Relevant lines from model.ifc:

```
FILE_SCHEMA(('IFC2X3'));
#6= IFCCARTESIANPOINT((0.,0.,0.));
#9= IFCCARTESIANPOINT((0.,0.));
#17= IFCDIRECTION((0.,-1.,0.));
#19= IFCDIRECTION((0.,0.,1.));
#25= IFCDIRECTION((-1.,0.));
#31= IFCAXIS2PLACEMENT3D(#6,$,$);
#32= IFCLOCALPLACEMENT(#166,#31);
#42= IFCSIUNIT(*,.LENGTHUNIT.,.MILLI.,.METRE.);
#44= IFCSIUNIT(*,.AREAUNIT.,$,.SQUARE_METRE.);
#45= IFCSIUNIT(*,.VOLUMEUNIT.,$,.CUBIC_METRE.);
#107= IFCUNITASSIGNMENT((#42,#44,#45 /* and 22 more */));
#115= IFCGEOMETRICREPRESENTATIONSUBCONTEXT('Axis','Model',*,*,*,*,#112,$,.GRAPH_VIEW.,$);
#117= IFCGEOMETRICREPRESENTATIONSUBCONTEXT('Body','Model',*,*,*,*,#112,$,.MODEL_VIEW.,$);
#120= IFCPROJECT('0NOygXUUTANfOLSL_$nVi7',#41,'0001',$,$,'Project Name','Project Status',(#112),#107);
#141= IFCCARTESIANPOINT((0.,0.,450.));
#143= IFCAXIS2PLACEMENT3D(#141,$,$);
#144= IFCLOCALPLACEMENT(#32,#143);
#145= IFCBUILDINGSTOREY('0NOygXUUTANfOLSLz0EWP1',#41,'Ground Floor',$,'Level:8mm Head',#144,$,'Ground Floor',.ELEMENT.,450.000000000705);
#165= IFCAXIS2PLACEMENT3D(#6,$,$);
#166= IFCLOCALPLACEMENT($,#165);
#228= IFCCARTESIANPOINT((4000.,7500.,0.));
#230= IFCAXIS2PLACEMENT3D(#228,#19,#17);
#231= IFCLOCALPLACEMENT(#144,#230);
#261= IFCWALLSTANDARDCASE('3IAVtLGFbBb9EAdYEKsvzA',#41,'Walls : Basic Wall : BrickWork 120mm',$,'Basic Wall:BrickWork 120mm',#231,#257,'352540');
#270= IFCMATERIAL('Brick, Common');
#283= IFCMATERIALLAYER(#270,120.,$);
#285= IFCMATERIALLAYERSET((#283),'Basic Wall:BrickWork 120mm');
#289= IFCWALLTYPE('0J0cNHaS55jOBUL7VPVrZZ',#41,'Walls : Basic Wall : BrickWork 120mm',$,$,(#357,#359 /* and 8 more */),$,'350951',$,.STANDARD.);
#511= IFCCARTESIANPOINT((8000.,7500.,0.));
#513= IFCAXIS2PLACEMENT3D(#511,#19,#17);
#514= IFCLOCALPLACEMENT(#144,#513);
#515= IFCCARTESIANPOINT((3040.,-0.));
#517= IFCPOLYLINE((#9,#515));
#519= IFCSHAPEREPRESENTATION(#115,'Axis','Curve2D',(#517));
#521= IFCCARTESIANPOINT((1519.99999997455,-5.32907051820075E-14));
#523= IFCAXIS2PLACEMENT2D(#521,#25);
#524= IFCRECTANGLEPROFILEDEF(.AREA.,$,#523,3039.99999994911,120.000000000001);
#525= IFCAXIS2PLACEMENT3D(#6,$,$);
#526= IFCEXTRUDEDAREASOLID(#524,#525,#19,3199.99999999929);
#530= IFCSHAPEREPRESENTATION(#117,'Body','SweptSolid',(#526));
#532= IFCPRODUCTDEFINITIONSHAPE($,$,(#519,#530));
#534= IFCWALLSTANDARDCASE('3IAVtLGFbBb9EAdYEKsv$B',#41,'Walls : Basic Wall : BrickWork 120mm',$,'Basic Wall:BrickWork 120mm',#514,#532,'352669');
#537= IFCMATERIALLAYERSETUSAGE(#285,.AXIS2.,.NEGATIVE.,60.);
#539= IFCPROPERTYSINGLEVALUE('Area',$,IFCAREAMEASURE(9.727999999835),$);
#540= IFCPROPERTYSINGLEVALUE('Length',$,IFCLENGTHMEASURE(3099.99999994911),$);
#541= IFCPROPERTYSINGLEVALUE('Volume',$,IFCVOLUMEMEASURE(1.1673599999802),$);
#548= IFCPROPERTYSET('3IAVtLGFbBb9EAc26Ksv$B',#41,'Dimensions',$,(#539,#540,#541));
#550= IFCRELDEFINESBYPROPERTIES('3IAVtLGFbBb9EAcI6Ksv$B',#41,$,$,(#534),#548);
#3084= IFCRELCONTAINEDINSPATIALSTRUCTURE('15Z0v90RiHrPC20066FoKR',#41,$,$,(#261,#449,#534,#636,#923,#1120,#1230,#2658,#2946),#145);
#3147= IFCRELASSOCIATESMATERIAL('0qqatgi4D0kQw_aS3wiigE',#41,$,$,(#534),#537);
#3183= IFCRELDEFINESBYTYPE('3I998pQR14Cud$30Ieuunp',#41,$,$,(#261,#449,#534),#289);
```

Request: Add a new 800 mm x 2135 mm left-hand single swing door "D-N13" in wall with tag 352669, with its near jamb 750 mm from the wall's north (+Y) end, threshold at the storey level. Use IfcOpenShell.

```python
import numpy as np
import ifcopenshell
import ifcopenshell.api.feature
import ifcopenshell.api.geometry
import ifcopenshell.api.pset
import ifcopenshell.api.root
import ifcopenshell.api.spatial
import ifcopenshell.api.type
import ifcopenshell.geom
import ifcopenshell.util.element
import ifcopenshell.util.placement
import ifcopenshell.util.representation
import ifcopenshell.util.shape
import ifcopenshell.util.unit

model = ifcopenshell.open("model.ifc")
unit_scale = ifcopenshell.util.unit.calculate_unit_scale(model)
area_scale = ifcopenshell.util.unit.calculate_unit_scale(model, "AREAUNIT")
volume_scale = ifcopenshell.util.unit.calculate_unit_scale(model, "VOLUMEUNIT")
settings = ifcopenshell.geom.settings()


def volume(element):
    """Net volume in cubic metres, openings subtracted."""
    shape = ifcopenshell.geom.create_shape(settings, element)
    return ifcopenshell.util.shape.get_volume(shape.geometry)


wall = model.by_guid("3IAVtLGFbBb9EAdYEKsv$B")
storey = ifcopenshell.util.element.get_container(wall, ifc_class="IfcBuildingStorey")
context = ifcopenshell.util.representation.get_context(model, "Model", "Body", "MODEL_VIEW")
before = volume(wall)

width, height, from_end, sill = 0.8, 2.135, 0.75, 0.0  # metres

# The wall runs along its own X axis, and the end named is its -X end.
wall_shape = ifcopenshell.geom.create_shape(settings, wall)
x, y, z = ifcopenshell.util.shape.get_vertices(wall_shape.geometry).T
start = x.min() + from_end
face, thickness = float(y.min()), float(y.max() - y.min())
wall_matrix = ifcopenshell.util.placement.get_local_placement(wall.ObjectPlacement)
level = ifcopenshell.util.placement.get_local_placement(storey.ObjectPlacement)[2, 3]


def in_wall(x, y):
    """Placement at x, y metres in the wall's axes, at sill height."""
    matrix = wall_matrix.copy()
    matrix[:, 3] = wall_matrix @ np.array([x / unit_scale, y / unit_scale, 0.0, 1.0])
    matrix[2, 3] = level + sill / unit_scale
    return matrix


# Opening: a box that overshoots both wall faces by 50 mm.
opening = ifcopenshell.api.root.create_entity(model, ifc_class="IfcOpeningElement")
box = ifcopenshell.api.geometry.add_wall_representation(
    model, context=context, length=width, height=height, thickness=thickness + 0.1
)
ifcopenshell.api.geometry.assign_representation(model, product=opening, representation=box)
ifcopenshell.api.geometry.edit_object_placement(model, product=opening, matrix=in_wall(start, face - 0.05), is_si=False)
ifcopenshell.api.feature.add_feature(model, feature=opening, element=wall)

door = ifcopenshell.api.root.create_entity(model, ifc_class="IfcDoor", name="D-N13")
door.OverallWidth, door.OverallHeight = width / unit_scale, height / unit_scale
body = ifcopenshell.api.geometry.add_door_representation(
    model,
    context=context,
    overall_width=door.OverallWidth,
    overall_height=door.OverallHeight,
    operation_type="SINGLE_SWING_LEFT",
    lining_properties={"LiningDepth": thickness / unit_scale, "ThresholdDepth": thickness / unit_scale},
)
ifcopenshell.api.geometry.assign_representation(model, product=door, representation=body)
ifcopenshell.api.spatial.assign_container(model, products=[door], relating_structure=storey)
fills = ifcopenshell.api.feature.add_filling(model, opening=opening, element=door)
fills.OwnerHistory = door.OwnerHistory  # required in IFC2X3

# IFC2X3 keeps the operation on the door style.
style = ifcopenshell.api.root.create_entity(model, ifc_class="IfcDoorStyle", name="D-N13")
style.OperationType, style.ConstructionType = "SINGLE_SWING_LEFT", "NOTDEFINED"
style.ParameterTakesPrecedence = style.Sizeable = False
ifcopenshell.api.type.assign_type(model, related_objects=[door], relating_type=style)

# The lining spans the wall, so the door starts at the wall face.
ifcopenshell.api.geometry.edit_object_placement(model, product=door, matrix=in_wall(start, face), is_si=False)

after = volume(wall)

# Update the wall's stored quantities.
pset = model.by_id(ifcopenshell.util.element.get_pset(wall, "Dimensions", should_inherit=False)["id"])
ifcopenshell.api.pset.edit_pset(model, pset=pset, properties={
    "Area": model.create_entity("IfcAreaMeasure", after / thickness / area_scale),
    "Volume": model.create_entity("IfcVolumeMeasure", after / volume_scale),
})

print(f"wall volume {before:.3f} -> {after:.3f} m3")

model.write("model-out.ifc")
```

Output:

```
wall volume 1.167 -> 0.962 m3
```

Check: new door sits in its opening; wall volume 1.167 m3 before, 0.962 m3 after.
